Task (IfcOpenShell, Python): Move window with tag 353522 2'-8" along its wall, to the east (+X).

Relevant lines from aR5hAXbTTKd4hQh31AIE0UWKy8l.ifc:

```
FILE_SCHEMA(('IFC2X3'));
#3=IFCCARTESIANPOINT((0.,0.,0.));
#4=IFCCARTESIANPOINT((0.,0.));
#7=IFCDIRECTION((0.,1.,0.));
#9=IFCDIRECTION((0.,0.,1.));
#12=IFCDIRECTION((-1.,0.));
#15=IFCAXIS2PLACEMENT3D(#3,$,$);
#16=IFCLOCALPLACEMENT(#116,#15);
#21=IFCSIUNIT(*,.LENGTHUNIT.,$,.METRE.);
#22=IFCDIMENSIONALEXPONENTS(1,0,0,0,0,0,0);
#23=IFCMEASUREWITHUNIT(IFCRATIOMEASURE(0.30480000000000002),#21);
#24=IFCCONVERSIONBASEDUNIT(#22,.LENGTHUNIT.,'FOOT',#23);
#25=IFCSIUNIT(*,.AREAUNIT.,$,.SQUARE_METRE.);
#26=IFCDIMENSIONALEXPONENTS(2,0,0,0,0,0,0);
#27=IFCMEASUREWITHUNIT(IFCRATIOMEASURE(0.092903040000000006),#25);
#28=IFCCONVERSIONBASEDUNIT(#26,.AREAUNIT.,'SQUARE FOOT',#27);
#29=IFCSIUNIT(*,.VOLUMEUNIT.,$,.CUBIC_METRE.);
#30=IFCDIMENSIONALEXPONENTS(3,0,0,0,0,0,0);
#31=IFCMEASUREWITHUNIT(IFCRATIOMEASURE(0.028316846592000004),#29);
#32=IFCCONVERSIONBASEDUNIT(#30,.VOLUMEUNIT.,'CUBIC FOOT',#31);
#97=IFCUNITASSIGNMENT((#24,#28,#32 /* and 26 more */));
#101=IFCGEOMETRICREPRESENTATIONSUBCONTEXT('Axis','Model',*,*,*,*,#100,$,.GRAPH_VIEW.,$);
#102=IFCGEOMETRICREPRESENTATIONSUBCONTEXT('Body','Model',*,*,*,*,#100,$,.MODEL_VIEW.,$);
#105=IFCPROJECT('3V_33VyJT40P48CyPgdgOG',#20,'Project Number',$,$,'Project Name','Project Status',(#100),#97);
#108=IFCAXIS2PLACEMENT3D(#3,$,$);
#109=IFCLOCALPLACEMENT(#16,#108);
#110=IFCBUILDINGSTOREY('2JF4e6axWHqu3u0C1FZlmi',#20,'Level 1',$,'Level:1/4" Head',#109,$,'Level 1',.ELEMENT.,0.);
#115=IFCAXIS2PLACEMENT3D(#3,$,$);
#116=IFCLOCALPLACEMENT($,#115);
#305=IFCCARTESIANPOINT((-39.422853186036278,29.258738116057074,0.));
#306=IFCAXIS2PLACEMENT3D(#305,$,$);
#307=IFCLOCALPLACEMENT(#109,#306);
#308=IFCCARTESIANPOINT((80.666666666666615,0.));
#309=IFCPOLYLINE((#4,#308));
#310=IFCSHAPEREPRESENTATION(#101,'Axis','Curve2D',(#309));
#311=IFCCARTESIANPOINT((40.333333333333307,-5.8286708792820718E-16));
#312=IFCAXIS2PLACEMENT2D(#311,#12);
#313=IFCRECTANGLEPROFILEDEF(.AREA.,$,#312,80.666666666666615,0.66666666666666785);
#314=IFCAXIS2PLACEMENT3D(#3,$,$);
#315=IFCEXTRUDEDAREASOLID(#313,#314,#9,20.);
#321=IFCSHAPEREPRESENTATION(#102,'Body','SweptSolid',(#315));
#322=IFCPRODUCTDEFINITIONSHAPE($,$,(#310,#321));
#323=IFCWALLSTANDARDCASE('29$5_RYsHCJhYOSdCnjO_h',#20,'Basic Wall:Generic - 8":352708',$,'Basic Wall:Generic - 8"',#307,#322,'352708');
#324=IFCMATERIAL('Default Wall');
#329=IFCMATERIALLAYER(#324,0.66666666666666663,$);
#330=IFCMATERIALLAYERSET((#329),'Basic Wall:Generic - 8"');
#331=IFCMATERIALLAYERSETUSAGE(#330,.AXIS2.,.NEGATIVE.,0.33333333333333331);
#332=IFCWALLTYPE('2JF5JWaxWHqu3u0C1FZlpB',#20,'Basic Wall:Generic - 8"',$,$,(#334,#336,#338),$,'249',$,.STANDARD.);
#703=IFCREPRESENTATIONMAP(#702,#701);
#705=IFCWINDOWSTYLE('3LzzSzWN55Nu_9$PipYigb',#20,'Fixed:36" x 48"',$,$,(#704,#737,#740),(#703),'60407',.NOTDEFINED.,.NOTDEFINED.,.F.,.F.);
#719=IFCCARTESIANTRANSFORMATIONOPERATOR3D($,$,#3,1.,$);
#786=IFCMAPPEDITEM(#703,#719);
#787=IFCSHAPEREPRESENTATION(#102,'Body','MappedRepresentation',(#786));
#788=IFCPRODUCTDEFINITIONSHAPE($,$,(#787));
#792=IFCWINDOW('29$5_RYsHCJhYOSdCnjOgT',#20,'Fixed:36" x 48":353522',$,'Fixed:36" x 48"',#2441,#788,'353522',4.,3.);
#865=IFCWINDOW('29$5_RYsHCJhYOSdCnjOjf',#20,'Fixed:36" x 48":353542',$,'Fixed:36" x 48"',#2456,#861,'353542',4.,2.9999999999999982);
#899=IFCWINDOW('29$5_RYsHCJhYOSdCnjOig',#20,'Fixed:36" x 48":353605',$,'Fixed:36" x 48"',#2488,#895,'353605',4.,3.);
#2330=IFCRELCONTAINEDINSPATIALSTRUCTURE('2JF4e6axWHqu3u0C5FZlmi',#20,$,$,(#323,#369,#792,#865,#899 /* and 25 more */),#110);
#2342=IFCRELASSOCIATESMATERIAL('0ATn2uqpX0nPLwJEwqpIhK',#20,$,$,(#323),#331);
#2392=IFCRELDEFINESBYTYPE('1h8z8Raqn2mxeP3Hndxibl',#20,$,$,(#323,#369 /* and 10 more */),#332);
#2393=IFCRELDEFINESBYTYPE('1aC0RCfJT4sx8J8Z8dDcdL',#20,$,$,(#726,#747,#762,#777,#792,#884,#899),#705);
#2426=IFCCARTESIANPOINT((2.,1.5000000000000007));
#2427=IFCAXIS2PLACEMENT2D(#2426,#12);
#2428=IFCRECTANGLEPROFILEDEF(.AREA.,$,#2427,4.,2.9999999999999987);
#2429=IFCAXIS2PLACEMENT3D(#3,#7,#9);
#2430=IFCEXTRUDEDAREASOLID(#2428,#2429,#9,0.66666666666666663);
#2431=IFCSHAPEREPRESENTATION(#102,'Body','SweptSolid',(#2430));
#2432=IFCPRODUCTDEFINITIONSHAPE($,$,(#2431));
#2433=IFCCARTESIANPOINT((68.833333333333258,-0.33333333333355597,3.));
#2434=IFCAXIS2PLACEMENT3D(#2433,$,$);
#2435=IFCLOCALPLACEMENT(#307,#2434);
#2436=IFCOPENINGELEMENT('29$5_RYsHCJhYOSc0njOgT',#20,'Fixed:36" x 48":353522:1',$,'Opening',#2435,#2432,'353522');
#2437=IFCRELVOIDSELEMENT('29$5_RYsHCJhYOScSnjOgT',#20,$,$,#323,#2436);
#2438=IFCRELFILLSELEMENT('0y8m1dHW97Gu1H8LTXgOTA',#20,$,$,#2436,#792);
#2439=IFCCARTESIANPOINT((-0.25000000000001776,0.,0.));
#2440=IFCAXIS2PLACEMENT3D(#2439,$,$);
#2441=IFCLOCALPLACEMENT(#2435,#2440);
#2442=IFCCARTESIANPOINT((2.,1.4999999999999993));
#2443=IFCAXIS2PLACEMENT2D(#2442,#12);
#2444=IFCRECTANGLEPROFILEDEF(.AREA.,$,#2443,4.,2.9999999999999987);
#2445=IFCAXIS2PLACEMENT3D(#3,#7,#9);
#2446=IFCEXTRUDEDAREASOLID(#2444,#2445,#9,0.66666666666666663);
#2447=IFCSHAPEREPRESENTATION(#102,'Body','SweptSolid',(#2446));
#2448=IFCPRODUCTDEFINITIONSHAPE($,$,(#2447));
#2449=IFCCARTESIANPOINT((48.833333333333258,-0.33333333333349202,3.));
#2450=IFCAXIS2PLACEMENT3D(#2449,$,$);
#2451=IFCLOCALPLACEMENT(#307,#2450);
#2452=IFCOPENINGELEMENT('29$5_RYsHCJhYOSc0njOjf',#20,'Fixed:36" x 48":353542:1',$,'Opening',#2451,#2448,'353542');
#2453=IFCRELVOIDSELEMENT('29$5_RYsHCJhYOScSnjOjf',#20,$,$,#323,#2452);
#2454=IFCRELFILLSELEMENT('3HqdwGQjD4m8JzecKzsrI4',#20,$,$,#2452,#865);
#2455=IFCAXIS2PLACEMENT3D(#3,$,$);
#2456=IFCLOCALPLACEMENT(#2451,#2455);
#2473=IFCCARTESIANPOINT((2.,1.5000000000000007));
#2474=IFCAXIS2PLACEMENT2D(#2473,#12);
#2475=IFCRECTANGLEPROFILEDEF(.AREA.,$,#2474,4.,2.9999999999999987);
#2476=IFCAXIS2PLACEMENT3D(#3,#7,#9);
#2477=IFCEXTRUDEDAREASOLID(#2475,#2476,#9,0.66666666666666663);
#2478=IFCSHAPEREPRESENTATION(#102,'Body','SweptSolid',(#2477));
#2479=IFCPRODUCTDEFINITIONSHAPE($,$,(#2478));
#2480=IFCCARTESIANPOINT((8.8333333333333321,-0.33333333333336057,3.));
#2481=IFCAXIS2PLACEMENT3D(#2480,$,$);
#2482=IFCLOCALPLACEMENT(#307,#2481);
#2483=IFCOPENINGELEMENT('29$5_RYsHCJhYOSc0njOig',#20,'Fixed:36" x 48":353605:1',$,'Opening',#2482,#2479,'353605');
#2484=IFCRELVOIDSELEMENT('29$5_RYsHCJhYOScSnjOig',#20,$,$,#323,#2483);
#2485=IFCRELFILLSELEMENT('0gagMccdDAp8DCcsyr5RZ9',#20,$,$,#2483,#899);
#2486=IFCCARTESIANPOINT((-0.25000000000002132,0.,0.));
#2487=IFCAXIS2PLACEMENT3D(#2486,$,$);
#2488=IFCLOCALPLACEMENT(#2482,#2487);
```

```python
import ifcopenshell
import ifcopenshell.api.geometry
import ifcopenshell.util.placement
import ifcopenshell.util.unit

model = ifcopenshell.open("aR5hAXbTTKd4hQh31AIE0UWKy8l.ifc")
unit_scale = ifcopenshell.util.unit.calculate_unit_scale(model)

window = model.by_guid("29$5_RYsHCJhYOSdCnjOgT")
opening = window.FillsVoids[0].RelatingOpeningElement
wall = opening.VoidsElements[0].RelatingBuildingElement

wall_matrix = ifcopenshell.util.placement.get_local_placement(wall.ObjectPlacement)
shift = wall_matrix[:3, 0] * 32 * 0.0254 / unit_scale
before = ifcopenshell.util.placement.get_local_placement(window.ObjectPlacement)[:3, 3].copy()

# The window is placed relative to its opening, so it follows when the opening moves.
matrix = ifcopenshell.util.placement.get_local_placement(opening.ObjectPlacement)
matrix[:3, 3] += shift
ifcopenshell.api.geometry.edit_object_placement(
    model, product=opening, matrix=matrix, is_si=False, should_transform_children=True
)

after = ifcopenshell.util.placement.get_local_placement(window.ObjectPlacement)[:3, 3]
print("window moved by", (after - before).round(3) + 0.0)

model.write("aR5hAXbTTKd4hQh31AIE0UWKy8l-out.ifc")
```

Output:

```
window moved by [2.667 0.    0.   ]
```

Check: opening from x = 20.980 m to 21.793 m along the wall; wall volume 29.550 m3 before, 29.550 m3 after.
